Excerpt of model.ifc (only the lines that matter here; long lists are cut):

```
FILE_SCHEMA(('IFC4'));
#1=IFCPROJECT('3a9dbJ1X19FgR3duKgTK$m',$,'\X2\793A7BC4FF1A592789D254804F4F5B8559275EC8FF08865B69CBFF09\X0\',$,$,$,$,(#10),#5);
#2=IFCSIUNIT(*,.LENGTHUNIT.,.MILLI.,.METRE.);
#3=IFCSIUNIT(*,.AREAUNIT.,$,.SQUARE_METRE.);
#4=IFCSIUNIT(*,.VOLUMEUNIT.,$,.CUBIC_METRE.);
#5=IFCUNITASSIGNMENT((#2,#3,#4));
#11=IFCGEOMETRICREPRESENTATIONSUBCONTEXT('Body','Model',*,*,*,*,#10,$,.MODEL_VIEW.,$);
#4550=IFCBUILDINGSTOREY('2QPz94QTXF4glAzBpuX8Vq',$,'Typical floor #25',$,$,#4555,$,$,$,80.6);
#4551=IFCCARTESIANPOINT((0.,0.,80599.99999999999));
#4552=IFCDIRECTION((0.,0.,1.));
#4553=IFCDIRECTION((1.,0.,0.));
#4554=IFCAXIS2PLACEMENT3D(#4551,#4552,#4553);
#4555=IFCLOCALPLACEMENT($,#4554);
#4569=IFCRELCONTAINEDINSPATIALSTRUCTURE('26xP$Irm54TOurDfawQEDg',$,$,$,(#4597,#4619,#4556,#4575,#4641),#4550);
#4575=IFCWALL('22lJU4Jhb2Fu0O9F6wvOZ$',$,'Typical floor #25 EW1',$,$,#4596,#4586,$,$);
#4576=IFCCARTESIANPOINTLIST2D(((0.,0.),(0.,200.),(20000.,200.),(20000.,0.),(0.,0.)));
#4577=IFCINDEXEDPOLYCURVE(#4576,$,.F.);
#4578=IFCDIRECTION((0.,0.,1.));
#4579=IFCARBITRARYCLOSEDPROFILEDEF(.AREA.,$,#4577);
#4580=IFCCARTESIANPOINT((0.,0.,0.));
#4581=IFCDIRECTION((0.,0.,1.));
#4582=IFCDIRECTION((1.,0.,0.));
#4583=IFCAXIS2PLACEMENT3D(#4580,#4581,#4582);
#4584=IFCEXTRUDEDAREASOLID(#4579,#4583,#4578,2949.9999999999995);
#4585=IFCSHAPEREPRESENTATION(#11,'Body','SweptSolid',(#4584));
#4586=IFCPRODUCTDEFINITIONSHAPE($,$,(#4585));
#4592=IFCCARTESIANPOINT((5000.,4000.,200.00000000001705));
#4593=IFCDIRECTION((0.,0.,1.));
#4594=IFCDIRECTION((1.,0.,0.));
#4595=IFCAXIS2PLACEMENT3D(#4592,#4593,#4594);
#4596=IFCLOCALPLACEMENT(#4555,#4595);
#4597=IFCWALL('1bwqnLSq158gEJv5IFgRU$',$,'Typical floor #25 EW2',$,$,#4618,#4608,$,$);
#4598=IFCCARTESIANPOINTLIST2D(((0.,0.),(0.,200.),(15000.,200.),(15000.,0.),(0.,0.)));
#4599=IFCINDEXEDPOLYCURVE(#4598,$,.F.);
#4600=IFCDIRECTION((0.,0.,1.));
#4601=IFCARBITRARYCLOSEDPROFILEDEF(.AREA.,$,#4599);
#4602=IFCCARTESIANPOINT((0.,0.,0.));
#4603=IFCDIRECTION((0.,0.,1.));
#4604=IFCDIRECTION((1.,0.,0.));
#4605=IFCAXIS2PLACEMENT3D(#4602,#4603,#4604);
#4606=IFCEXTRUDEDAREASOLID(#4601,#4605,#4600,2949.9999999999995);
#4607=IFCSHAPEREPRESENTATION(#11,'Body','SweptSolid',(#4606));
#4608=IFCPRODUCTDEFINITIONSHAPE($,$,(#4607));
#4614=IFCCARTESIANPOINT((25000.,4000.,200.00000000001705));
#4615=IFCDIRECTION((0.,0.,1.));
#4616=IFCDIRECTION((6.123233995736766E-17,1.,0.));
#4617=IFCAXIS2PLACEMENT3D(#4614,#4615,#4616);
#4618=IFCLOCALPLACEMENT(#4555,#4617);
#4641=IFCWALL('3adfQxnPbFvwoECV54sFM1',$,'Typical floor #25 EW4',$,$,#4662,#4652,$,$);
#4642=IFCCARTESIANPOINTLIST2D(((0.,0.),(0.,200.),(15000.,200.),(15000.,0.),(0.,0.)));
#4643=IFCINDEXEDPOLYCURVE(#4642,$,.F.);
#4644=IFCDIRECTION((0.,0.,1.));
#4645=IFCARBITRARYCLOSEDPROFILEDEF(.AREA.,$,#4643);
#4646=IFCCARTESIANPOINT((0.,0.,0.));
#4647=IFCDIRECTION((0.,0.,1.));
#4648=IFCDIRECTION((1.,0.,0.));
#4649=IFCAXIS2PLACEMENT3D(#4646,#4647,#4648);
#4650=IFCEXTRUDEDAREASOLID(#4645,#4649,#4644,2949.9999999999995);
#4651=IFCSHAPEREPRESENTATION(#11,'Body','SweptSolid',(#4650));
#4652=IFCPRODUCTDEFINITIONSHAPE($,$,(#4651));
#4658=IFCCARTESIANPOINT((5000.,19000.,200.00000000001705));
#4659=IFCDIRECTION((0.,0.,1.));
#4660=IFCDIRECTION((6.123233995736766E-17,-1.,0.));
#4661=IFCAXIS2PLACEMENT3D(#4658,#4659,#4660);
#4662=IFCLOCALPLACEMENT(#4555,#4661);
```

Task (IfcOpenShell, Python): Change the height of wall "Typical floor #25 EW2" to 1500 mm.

```python
import ifcopenshell
import ifcopenshell.geom
import ifcopenshell.util.representation
import ifcopenshell.util.shape

model = ifcopenshell.open("model.ifc")
settings = ifcopenshell.geom.settings()


def volume(element):
    """Net volume in cubic metres, openings subtracted."""
    shape = ifcopenshell.geom.create_shape(settings, element)
    return ifcopenshell.util.shape.get_volume(shape.geometry)


wall = model.by_guid("1bwqnLSq158gEJv5IFgRU$")
before = volume(wall)

body = ifcopenshell.util.representation.get_representation(wall, "Model", "Body")
solid = body.Items[0]
old_height = solid.Depth
solid.Depth = 1500.0
after = volume(wall)

print(f"height {old_height:g} -> {solid.Depth:g}, volume {before:.3f} -> {after:.3f} m3")

model.write("model_rev.ifc")
```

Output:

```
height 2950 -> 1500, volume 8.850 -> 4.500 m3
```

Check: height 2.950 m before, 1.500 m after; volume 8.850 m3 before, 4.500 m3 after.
